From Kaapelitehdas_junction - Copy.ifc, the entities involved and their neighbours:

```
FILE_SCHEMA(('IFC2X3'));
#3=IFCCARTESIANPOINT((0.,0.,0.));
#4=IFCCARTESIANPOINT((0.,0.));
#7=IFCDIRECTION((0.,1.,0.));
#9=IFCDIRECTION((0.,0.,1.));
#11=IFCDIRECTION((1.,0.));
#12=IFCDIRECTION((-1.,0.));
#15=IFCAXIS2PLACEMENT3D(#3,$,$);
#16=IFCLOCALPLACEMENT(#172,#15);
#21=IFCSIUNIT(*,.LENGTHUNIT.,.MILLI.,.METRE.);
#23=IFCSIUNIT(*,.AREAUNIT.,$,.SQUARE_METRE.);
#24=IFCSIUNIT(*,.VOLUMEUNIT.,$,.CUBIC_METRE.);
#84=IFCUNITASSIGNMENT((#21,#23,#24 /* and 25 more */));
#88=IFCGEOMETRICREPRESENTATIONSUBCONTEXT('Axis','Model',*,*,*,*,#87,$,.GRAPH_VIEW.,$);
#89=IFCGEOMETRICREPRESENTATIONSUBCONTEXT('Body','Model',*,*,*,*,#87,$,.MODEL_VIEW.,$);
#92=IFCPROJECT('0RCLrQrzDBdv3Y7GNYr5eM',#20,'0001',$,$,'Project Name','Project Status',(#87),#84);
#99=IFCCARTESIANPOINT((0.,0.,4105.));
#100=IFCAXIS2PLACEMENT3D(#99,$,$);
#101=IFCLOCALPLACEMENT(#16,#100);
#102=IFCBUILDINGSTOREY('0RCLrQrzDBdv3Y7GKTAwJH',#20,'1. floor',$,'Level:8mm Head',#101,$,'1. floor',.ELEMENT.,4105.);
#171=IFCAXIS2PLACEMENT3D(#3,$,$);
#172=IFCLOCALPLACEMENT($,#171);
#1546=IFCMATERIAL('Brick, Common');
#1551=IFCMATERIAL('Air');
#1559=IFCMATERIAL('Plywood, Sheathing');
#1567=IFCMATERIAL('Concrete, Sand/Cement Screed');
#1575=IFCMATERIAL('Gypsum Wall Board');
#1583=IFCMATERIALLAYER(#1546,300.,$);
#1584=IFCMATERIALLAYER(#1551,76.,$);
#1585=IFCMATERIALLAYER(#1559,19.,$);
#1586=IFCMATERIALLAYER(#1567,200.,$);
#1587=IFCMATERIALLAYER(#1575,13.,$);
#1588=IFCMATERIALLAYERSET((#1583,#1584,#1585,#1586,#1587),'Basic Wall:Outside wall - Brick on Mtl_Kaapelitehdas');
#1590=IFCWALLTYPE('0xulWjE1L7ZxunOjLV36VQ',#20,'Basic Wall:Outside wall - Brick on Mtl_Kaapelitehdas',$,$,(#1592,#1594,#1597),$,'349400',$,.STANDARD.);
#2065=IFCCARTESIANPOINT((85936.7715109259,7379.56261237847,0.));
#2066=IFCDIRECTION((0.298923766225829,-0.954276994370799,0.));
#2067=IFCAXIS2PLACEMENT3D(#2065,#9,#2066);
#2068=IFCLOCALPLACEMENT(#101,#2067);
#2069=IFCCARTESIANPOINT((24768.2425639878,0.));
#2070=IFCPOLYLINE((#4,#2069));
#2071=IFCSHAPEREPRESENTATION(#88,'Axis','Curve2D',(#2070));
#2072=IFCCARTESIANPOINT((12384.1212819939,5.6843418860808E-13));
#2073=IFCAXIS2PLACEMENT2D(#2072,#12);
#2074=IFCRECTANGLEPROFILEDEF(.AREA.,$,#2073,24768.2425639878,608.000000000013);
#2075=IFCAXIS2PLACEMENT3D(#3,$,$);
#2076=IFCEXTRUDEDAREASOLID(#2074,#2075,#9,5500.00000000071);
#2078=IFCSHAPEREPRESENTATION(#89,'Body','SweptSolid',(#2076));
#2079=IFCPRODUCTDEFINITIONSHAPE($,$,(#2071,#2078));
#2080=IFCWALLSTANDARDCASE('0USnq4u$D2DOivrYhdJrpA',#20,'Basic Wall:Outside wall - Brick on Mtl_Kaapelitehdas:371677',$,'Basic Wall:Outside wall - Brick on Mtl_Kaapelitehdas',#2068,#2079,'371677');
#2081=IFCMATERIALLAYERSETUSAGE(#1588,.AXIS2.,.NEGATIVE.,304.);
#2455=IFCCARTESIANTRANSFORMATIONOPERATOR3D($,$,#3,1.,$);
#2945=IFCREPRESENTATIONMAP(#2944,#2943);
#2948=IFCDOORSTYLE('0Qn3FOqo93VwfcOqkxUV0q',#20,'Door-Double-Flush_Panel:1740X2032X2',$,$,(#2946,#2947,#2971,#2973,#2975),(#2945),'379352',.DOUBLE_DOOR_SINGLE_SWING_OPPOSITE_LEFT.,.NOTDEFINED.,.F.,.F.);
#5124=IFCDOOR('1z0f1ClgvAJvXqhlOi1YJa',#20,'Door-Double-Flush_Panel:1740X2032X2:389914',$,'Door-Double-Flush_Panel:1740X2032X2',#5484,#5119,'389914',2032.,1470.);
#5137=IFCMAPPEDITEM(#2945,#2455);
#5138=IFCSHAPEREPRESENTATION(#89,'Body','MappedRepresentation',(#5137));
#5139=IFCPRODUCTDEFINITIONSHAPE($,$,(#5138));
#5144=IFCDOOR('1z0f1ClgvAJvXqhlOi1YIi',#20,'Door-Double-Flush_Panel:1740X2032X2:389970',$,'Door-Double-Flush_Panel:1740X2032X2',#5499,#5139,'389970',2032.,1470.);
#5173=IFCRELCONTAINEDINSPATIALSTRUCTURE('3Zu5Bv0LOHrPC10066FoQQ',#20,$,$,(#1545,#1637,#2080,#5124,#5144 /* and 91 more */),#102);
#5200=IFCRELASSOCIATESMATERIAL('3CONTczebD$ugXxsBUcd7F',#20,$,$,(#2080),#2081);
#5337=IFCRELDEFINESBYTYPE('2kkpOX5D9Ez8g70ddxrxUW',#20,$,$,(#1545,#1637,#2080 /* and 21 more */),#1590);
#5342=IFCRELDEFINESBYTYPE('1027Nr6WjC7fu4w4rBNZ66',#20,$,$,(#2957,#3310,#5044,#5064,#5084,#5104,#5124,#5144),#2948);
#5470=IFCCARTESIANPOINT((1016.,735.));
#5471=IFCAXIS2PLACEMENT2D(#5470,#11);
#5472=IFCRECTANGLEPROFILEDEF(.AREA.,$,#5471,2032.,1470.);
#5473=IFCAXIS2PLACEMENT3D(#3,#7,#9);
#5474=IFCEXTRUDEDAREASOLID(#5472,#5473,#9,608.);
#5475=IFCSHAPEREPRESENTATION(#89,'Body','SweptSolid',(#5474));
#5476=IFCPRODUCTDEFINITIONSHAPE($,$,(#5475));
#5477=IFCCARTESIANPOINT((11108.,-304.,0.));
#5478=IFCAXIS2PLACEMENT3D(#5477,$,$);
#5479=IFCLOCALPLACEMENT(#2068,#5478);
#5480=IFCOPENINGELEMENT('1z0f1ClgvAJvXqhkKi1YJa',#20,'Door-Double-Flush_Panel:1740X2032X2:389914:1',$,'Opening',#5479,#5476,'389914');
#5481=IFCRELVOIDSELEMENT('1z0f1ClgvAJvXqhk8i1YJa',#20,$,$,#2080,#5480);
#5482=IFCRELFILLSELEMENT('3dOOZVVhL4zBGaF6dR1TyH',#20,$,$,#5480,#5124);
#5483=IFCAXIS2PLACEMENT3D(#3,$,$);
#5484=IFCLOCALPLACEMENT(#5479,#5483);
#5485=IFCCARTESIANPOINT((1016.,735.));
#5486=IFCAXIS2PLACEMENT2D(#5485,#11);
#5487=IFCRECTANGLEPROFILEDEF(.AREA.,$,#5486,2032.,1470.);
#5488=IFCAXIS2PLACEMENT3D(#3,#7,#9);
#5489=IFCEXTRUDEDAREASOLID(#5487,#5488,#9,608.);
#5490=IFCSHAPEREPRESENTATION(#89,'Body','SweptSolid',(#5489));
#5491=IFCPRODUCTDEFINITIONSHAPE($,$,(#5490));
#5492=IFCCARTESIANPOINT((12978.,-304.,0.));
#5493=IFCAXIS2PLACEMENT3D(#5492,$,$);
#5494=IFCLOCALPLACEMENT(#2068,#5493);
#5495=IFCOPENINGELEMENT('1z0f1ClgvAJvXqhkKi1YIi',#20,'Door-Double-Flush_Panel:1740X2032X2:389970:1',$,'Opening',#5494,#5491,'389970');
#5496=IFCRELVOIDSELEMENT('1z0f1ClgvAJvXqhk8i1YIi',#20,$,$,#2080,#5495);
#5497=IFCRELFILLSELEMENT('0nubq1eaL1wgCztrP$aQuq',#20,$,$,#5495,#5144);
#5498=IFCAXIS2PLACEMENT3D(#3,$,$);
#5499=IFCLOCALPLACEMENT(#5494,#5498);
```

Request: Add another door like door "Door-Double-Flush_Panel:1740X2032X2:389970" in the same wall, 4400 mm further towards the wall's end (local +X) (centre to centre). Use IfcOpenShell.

```python
import ifcopenshell
import ifcopenshell.api.feature
import ifcopenshell.api.geometry
import ifcopenshell.api.root
import ifcopenshell.geom
import ifcopenshell.util.element
import ifcopenshell.util.placement
import ifcopenshell.util.shape
import ifcopenshell.util.unit

model = ifcopenshell.open("Kaapelitehdas_junction - Copy.ifc")
unit_scale = ifcopenshell.util.unit.calculate_unit_scale(model)
settings = ifcopenshell.geom.settings()


def volume(element):
    """Net volume in cubic metres, openings subtracted."""
    shape = ifcopenshell.geom.create_shape(settings, element)
    return ifcopenshell.util.shape.get_volume(shape.geometry)


def reuse_history(source, copy):
    """copy_class also copies each property set's owner history, people and application; keep the originals."""
    for rel in copy.IsDefinedBy:
        if rel.is_a("IfcRelDefinesByProperties") and (history := rel.RelatingPropertyDefinition.OwnerHistory):
            rel.RelatingPropertyDefinition.OwnerHistory = source.OwnerHistory
            ifcopenshell.util.element.remove_deep2(model, history)


door = model.by_guid("1z0f1ClgvAJvXqhlOi1YIi")
opening = door.FillsVoids[0].RelatingOpeningElement
wall = opening.VoidsElements[0].RelatingBuildingElement
before = volume(wall)
shift = ifcopenshell.util.placement.get_local_placement(wall.ObjectPlacement)[:3, 0] * 4.4 / unit_scale

# copy_class copies the void relationship, type, container and properties, but no geometry.
new_opening = ifcopenshell.api.root.copy_class(model, product=opening)
new_opening.Representation = ifcopenshell.util.element.copy_deep(
    model, opening.Representation, exclude=["IfcGeometricRepresentationContext", "IfcRepresentationMap"]
)
new_opening.Name = "Door-Double-Flush_Panel:1740X2032X2"
new_opening.Tag = None
new_door = ifcopenshell.api.root.copy_class(model, product=door)
new_door.Representation = ifcopenshell.util.element.copy_deep(
    model, door.Representation, exclude=["IfcGeometricRepresentationContext", "IfcRepresentationMap"]
)
new_door.Name = "Door-Double-Flush_Panel:1740X2032X2"
new_door.Tag = None
reuse_history(door, new_door)
fills = ifcopenshell.api.feature.add_filling(model, opening=new_opening, element=new_door)
fills.OwnerHistory = new_door.OwnerHistory  # required in IFC2X3

for old, new in ((opening, new_opening), (door, new_door)):
    matrix = ifcopenshell.util.placement.get_local_placement(old.ObjectPlacement)
    matrix[:3, 3] += shift
    ifcopenshell.api.geometry.edit_object_placement(model, product=new, matrix=matrix, is_si=False)

after = volume(wall)

print(f"wall volume {before:.3f} -> {after:.3f} m3")

model.write("Kaapelitehdas_junction - Copy_updated.ifc")
```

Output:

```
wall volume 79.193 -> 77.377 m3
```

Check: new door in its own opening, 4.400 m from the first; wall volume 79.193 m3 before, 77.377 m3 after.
